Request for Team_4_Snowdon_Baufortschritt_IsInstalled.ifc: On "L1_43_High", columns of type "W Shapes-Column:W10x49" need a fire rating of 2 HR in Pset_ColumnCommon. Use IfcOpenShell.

First a look at what the model holds.

```python
import ifcopenshell
import ifcopenshell.util.element

model = ifcopenshell.open("Team_4_Snowdon_Baufortschritt_IsInstalled.ifc")
print(model.schema)
storey = next(s for s in model.by_type("IfcBuildingStorey") if s.Name == "L1_43_High")
columns = [e for e in ifcopenshell.util.element.get_decomposition(storey) if e.is_a("IfcColumn")]
seen = {}
for e in columns:
    element_type = ifcopenshell.util.element.get_type(e)
    key = (element_type.Name if element_type != e and element_type else None, ifcopenshell.util.element.get_pset(e, "Pset_ColumnCommon", "FireRating"))
    seen[key] = seen.get(key, 0) + 1
for (name, value), count in sorted(seen.items(), key=str):
    print(count, "x", name, "|", value)
```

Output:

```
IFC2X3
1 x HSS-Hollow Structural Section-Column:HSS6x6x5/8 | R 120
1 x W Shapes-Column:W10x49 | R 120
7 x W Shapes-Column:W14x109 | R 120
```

```python
import ifcopenshell
import ifcopenshell.api.pset
import ifcopenshell.util.element

model = ifcopenshell.open("Team_4_Snowdon_Baufortschritt_IsInstalled.ifc")

storey = next(s for s in model.by_type("IfcBuildingStorey") if s.Name == "L1_43_High")
columns = [e for e in ifcopenshell.util.element.get_decomposition(storey) if e.is_a("IfcColumn")]

count = 0
for e in columns:
    element_type = ifcopenshell.util.element.get_type(e)
    if element_type in (None, e) or element_type.Name != "W Shapes-Column:W10x49":
        continue
    # add_pset returns the element's existing set when there is one.
    pset = ifcopenshell.api.pset.add_pset(model, product=e, name="Pset_ColumnCommon")
    ifcopenshell.api.pset.edit_pset(model, pset=pset, properties={"FireRating": "2 HR"})
    count += 1

print(count, "columns updated")

model.write("Team_4_Snowdon_Baufortschritt_IsInstalled_edited.ifc")
```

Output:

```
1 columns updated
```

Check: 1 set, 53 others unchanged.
